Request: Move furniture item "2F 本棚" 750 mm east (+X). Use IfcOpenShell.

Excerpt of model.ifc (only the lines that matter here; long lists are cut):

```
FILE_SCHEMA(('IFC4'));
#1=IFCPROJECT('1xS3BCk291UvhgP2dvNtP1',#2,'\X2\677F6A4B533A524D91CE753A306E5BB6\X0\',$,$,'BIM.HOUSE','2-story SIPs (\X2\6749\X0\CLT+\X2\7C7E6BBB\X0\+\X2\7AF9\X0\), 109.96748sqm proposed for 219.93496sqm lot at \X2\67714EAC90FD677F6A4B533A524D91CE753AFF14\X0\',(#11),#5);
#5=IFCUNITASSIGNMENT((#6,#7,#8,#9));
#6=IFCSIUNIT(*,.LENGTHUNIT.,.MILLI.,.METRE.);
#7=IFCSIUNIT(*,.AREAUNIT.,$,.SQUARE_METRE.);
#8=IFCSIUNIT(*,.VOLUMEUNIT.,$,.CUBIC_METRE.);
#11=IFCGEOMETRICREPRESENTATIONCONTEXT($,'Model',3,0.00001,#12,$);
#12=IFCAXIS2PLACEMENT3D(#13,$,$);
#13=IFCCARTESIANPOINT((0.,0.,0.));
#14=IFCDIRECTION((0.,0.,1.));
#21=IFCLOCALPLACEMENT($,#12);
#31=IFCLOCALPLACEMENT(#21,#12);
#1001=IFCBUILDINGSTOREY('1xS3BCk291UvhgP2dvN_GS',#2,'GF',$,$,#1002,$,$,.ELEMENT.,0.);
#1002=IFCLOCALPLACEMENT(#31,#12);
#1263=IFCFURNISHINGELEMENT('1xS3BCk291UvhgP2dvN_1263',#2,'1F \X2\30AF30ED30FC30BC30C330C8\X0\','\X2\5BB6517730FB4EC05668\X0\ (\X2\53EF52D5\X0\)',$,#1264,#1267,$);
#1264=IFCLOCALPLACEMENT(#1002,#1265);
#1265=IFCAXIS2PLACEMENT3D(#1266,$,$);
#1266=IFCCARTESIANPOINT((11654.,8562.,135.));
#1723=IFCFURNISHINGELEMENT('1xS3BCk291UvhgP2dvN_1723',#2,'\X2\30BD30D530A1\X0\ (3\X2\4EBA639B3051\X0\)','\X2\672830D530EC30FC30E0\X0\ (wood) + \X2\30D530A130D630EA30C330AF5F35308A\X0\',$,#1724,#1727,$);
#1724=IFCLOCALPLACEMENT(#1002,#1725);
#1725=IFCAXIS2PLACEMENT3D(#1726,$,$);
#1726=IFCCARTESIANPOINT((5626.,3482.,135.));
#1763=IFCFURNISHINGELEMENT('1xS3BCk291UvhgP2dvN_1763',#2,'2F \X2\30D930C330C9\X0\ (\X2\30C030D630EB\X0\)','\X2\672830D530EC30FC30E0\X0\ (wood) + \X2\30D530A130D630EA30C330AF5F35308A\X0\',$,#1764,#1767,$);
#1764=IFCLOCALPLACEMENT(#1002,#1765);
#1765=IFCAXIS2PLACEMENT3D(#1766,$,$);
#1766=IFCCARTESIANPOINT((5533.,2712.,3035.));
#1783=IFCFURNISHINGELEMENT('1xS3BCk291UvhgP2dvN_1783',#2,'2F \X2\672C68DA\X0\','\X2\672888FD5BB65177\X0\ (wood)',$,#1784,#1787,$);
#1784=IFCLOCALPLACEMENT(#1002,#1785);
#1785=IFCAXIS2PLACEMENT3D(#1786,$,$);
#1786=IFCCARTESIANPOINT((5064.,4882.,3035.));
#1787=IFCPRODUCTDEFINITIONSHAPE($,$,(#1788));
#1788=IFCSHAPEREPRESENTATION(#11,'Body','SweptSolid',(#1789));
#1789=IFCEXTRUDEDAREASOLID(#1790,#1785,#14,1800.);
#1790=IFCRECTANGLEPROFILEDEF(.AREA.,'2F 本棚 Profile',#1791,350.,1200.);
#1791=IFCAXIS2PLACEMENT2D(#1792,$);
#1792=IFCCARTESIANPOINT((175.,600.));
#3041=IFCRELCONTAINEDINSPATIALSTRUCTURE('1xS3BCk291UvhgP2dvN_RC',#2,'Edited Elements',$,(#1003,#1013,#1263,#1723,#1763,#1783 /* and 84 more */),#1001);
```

```python
import ifcopenshell
import ifcopenshell.api.geometry
import ifcopenshell.util.placement
import ifcopenshell.util.unit

model = ifcopenshell.open("model.ifc")
unit_scale = ifcopenshell.util.unit.calculate_unit_scale(model)

item = model.by_id(1783)
matrix = ifcopenshell.util.placement.get_local_placement(item.ObjectPlacement)
matrix[0, 3] += 0.75 / unit_scale
ifcopenshell.api.geometry.edit_object_placement(model, product=item, matrix=matrix, is_si=False)

print(ifcopenshell.util.placement.get_local_placement(item.ObjectPlacement).round(3) + 0.0)

model.write("model-out.ifc")
```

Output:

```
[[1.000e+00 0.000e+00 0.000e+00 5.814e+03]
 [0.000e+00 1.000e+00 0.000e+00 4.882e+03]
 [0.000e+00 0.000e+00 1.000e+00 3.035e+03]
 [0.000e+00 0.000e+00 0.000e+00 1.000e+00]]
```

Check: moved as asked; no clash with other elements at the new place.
